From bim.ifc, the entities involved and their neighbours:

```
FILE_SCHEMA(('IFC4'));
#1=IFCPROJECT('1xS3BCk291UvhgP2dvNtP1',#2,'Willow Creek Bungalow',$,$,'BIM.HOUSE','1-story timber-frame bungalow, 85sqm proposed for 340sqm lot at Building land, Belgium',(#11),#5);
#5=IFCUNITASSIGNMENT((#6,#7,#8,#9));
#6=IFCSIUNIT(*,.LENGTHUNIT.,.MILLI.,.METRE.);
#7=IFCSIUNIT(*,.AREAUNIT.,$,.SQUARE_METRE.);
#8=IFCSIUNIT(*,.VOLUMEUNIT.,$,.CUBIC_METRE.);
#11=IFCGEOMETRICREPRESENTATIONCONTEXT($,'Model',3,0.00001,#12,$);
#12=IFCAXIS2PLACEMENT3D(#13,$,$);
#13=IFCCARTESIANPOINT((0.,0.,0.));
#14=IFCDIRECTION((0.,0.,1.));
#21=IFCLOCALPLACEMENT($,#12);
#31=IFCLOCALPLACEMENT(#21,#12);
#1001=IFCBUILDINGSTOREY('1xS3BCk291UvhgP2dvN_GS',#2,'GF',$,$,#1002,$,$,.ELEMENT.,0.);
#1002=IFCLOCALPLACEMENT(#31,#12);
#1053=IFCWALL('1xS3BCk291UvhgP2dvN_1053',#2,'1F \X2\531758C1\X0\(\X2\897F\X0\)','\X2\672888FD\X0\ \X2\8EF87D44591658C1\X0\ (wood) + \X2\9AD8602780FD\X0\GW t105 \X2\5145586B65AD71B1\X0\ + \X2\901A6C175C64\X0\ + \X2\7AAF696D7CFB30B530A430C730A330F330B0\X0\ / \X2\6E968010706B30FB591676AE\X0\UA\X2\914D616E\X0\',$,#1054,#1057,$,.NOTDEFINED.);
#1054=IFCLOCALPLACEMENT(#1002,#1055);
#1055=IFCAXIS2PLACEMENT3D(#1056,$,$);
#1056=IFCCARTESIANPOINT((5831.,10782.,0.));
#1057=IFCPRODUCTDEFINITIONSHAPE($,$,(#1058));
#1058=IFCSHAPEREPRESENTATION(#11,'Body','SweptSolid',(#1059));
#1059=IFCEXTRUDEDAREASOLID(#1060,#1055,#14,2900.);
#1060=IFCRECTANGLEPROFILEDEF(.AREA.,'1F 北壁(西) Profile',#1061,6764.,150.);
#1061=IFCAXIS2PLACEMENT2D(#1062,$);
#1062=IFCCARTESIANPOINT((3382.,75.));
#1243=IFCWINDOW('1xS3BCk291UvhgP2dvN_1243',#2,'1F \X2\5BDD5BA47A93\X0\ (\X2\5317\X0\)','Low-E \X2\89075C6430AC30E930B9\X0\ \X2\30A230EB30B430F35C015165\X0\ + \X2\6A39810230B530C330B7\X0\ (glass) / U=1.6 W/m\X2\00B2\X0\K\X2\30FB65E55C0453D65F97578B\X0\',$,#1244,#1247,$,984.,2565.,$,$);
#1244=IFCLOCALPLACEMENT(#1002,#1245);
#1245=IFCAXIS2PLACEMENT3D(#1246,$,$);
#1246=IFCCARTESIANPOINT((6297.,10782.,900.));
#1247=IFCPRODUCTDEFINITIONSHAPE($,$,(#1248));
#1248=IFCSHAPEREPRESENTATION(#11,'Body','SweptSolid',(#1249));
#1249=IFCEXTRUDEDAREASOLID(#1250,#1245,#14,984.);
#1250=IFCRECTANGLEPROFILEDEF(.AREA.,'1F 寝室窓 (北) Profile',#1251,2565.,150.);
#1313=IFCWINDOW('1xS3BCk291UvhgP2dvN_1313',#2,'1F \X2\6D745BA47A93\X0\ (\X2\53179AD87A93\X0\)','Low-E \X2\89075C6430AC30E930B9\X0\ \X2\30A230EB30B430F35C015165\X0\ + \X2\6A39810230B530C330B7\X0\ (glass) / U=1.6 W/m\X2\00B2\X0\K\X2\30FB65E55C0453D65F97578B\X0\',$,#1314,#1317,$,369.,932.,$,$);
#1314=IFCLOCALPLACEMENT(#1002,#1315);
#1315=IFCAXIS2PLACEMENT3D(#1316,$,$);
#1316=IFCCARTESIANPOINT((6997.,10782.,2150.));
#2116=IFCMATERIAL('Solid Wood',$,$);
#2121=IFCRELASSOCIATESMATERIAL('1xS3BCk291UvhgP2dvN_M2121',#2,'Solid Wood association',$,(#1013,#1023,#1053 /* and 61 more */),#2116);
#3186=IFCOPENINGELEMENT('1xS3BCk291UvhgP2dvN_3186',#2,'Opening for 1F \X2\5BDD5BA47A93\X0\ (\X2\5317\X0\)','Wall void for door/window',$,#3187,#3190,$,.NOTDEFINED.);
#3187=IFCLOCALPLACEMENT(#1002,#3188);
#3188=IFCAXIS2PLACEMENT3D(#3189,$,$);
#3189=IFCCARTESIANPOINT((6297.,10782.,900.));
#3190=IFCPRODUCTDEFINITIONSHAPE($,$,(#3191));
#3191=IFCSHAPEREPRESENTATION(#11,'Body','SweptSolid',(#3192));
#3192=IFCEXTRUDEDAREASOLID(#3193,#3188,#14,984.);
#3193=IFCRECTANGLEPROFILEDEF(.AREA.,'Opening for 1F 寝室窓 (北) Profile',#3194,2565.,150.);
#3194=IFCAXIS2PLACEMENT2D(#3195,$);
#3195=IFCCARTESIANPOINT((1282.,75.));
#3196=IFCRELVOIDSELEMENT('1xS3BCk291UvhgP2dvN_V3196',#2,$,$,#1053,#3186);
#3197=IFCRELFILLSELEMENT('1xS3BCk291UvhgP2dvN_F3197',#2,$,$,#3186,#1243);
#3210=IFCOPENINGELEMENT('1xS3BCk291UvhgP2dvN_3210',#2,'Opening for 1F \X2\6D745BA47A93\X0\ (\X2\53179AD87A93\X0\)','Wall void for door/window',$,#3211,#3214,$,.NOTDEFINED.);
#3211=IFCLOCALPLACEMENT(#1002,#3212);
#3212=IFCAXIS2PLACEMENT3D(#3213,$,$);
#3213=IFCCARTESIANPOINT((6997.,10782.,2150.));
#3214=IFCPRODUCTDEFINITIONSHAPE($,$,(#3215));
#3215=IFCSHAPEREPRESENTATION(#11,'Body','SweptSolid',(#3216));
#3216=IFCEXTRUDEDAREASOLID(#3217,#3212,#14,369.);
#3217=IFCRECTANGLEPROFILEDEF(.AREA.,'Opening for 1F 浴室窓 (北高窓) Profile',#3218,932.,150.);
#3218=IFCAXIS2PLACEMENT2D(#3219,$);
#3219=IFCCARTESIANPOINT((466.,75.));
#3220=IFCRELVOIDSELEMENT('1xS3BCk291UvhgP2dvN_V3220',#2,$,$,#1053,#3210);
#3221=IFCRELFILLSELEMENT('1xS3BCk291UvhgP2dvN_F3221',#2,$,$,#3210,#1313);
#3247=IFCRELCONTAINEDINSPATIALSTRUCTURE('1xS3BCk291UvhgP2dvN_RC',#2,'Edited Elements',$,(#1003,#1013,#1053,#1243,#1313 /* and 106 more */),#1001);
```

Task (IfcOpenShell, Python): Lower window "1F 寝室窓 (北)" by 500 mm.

```python
import numpy as np
import ifcopenshell
import ifcopenshell.api.geometry
import ifcopenshell.util.placement
import ifcopenshell.util.unit

model = ifcopenshell.open("bim.ifc")
unit_scale = ifcopenshell.util.unit.calculate_unit_scale(model)

window = model.by_guid("1xS3BCk291UvhgP2dvN_1243")
opening = window.FillsVoids[0].RelatingOpeningElement
dz = -500.0

shift = np.array([0.0, 0.0, dz])
# The window is not placed relative to its opening, so move both.
for product in (opening, window):
    matrix = ifcopenshell.util.placement.get_local_placement(product.ObjectPlacement)
    matrix[:3, 3] += shift
    ifcopenshell.api.geometry.edit_object_placement(model, product=product, matrix=matrix, is_si=False)

print(f"moved by {dz * unit_scale:+.3f} m")

model.write("bim_updated.ifc")
```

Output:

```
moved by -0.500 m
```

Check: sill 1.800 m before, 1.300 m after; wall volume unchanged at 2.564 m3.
